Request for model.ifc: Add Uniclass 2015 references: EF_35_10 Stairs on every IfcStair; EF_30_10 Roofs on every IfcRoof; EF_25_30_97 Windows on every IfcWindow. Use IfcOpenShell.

First a look at what the model holds.

```python
import ifcopenshell

model = ifcopenshell.open("model.ifc")
print(model.schema)
print("classifications:", [c.Name for c in model.by_type("IfcClassification")])
for ifc_class in ("IfcDoor", "IfcRoof", "IfcStair", "IfcWall", "IfcWindow"):
    print(ifc_class, len(model.by_type(ifc_class)))
```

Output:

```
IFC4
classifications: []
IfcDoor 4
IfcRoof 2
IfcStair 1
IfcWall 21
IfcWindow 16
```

```python
import ifcopenshell
import ifcopenshell.api.classification

model = ifcopenshell.open("model.ifc")

system = ifcopenshell.api.classification.add_classification(model, classification="Uniclass 2015")

codes = {
    "IfcStair": ("EF_35_10", "Stairs"),
    "IfcRoof": ("EF_30_10", "Roofs"),
    "IfcWindow": ("EF_25_30_97", "Windows"),
}
for ifc_class, (code, name) in codes.items():
    products = model.by_type(ifc_class)
    ifcopenshell.api.classification.add_reference(
        model, products=products, classification=system, identification=code, name=name
    )
    print(code, len(products))

model.write("model-out.ifc")
```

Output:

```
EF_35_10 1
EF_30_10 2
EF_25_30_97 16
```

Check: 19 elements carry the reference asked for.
